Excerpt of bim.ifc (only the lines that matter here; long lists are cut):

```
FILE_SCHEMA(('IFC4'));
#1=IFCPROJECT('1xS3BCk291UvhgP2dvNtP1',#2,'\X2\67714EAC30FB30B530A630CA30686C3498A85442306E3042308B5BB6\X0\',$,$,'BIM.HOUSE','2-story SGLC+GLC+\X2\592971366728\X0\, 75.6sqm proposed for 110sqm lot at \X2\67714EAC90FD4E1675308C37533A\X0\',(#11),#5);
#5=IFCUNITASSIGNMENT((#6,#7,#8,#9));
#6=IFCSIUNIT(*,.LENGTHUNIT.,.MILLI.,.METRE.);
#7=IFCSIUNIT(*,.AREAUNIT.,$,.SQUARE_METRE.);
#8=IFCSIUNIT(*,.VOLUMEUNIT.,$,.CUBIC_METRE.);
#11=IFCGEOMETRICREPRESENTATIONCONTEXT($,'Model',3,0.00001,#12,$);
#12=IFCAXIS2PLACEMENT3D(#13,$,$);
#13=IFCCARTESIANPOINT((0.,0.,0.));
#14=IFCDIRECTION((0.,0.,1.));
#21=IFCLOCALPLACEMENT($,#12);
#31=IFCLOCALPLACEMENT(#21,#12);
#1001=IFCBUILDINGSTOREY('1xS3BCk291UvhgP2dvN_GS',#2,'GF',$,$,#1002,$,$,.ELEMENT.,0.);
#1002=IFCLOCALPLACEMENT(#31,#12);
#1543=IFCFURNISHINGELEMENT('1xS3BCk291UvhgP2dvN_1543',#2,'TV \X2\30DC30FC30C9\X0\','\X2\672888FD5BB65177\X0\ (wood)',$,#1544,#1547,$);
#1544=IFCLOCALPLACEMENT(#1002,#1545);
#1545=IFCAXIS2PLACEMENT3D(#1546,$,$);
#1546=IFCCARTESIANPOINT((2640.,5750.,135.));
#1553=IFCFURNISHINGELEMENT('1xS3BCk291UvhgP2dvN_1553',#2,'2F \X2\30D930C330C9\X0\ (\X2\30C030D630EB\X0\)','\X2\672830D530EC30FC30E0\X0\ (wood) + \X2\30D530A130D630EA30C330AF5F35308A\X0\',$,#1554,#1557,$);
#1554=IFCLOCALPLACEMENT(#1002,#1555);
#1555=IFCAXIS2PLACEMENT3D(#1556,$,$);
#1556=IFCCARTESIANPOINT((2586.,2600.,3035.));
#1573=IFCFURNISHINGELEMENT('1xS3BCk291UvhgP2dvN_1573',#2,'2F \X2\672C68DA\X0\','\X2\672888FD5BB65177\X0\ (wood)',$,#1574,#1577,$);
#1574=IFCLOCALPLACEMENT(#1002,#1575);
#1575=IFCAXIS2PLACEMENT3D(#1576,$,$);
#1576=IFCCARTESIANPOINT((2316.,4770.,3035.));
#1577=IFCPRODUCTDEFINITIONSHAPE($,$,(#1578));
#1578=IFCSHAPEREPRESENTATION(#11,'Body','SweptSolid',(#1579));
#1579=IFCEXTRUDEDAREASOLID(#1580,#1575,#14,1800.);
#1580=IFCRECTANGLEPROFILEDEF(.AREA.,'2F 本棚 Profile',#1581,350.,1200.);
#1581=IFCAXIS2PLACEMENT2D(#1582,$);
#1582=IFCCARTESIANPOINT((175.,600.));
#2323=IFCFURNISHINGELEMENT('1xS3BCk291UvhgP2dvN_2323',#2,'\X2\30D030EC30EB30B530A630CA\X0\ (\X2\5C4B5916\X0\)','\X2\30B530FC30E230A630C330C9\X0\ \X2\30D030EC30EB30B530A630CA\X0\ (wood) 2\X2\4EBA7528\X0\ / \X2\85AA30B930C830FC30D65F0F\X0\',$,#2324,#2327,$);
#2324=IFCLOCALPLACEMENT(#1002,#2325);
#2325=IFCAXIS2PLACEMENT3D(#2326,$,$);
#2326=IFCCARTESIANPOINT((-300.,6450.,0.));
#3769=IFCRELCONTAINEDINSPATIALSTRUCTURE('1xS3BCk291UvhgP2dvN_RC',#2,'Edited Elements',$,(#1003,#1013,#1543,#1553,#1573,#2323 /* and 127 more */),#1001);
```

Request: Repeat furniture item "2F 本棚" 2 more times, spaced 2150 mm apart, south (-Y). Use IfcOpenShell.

```python
import numpy as np
import ifcopenshell
import ifcopenshell.api.geometry
import ifcopenshell.api.root
import ifcopenshell.util.element
import ifcopenshell.util.placement
import ifcopenshell.util.unit

model = ifcopenshell.open("bim.ifc")
unit_scale = ifcopenshell.util.unit.calculate_unit_scale(model)


def reuse_history(source, copy):
    """copy_class also copies each property set's owner history, people and application; keep the originals."""
    for rel in copy.IsDefinedBy:
        if rel.is_a("IfcRelDefinesByProperties") and (history := rel.RelatingPropertyDefinition.OwnerHistory):
            rel.RelatingPropertyDefinition.OwnerHistory = source.OwnerHistory
            ifcopenshell.util.element.remove_deep2(model, history)


source = model.by_guid("1xS3BCk291UvhgP2dvN_1573")
base = ifcopenshell.util.placement.get_local_placement(source.ObjectPlacement)
step = np.array([0.0, -1.0, 0.0]) * 2.15 / unit_scale

for i in range(1, 3):
    copy = ifcopenshell.api.root.copy_class(model, product=source)
    copy.Representation = ifcopenshell.util.element.copy_deep(
        model, source.Representation, exclude=["IfcGeometricRepresentationContext", "IfcRepresentationMap"]
    )
    reuse_history(source, copy)
    matrix = base.copy()
    matrix[:3, 3] += i * step
    print("added at", matrix[:3, 3].round(3) + 0.0)
    ifcopenshell.api.geometry.edit_object_placement(model, product=copy, matrix=matrix, is_si=False)

model.write("bim-out.ifc")
```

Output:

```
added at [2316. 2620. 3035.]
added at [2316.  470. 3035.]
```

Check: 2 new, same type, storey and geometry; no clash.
